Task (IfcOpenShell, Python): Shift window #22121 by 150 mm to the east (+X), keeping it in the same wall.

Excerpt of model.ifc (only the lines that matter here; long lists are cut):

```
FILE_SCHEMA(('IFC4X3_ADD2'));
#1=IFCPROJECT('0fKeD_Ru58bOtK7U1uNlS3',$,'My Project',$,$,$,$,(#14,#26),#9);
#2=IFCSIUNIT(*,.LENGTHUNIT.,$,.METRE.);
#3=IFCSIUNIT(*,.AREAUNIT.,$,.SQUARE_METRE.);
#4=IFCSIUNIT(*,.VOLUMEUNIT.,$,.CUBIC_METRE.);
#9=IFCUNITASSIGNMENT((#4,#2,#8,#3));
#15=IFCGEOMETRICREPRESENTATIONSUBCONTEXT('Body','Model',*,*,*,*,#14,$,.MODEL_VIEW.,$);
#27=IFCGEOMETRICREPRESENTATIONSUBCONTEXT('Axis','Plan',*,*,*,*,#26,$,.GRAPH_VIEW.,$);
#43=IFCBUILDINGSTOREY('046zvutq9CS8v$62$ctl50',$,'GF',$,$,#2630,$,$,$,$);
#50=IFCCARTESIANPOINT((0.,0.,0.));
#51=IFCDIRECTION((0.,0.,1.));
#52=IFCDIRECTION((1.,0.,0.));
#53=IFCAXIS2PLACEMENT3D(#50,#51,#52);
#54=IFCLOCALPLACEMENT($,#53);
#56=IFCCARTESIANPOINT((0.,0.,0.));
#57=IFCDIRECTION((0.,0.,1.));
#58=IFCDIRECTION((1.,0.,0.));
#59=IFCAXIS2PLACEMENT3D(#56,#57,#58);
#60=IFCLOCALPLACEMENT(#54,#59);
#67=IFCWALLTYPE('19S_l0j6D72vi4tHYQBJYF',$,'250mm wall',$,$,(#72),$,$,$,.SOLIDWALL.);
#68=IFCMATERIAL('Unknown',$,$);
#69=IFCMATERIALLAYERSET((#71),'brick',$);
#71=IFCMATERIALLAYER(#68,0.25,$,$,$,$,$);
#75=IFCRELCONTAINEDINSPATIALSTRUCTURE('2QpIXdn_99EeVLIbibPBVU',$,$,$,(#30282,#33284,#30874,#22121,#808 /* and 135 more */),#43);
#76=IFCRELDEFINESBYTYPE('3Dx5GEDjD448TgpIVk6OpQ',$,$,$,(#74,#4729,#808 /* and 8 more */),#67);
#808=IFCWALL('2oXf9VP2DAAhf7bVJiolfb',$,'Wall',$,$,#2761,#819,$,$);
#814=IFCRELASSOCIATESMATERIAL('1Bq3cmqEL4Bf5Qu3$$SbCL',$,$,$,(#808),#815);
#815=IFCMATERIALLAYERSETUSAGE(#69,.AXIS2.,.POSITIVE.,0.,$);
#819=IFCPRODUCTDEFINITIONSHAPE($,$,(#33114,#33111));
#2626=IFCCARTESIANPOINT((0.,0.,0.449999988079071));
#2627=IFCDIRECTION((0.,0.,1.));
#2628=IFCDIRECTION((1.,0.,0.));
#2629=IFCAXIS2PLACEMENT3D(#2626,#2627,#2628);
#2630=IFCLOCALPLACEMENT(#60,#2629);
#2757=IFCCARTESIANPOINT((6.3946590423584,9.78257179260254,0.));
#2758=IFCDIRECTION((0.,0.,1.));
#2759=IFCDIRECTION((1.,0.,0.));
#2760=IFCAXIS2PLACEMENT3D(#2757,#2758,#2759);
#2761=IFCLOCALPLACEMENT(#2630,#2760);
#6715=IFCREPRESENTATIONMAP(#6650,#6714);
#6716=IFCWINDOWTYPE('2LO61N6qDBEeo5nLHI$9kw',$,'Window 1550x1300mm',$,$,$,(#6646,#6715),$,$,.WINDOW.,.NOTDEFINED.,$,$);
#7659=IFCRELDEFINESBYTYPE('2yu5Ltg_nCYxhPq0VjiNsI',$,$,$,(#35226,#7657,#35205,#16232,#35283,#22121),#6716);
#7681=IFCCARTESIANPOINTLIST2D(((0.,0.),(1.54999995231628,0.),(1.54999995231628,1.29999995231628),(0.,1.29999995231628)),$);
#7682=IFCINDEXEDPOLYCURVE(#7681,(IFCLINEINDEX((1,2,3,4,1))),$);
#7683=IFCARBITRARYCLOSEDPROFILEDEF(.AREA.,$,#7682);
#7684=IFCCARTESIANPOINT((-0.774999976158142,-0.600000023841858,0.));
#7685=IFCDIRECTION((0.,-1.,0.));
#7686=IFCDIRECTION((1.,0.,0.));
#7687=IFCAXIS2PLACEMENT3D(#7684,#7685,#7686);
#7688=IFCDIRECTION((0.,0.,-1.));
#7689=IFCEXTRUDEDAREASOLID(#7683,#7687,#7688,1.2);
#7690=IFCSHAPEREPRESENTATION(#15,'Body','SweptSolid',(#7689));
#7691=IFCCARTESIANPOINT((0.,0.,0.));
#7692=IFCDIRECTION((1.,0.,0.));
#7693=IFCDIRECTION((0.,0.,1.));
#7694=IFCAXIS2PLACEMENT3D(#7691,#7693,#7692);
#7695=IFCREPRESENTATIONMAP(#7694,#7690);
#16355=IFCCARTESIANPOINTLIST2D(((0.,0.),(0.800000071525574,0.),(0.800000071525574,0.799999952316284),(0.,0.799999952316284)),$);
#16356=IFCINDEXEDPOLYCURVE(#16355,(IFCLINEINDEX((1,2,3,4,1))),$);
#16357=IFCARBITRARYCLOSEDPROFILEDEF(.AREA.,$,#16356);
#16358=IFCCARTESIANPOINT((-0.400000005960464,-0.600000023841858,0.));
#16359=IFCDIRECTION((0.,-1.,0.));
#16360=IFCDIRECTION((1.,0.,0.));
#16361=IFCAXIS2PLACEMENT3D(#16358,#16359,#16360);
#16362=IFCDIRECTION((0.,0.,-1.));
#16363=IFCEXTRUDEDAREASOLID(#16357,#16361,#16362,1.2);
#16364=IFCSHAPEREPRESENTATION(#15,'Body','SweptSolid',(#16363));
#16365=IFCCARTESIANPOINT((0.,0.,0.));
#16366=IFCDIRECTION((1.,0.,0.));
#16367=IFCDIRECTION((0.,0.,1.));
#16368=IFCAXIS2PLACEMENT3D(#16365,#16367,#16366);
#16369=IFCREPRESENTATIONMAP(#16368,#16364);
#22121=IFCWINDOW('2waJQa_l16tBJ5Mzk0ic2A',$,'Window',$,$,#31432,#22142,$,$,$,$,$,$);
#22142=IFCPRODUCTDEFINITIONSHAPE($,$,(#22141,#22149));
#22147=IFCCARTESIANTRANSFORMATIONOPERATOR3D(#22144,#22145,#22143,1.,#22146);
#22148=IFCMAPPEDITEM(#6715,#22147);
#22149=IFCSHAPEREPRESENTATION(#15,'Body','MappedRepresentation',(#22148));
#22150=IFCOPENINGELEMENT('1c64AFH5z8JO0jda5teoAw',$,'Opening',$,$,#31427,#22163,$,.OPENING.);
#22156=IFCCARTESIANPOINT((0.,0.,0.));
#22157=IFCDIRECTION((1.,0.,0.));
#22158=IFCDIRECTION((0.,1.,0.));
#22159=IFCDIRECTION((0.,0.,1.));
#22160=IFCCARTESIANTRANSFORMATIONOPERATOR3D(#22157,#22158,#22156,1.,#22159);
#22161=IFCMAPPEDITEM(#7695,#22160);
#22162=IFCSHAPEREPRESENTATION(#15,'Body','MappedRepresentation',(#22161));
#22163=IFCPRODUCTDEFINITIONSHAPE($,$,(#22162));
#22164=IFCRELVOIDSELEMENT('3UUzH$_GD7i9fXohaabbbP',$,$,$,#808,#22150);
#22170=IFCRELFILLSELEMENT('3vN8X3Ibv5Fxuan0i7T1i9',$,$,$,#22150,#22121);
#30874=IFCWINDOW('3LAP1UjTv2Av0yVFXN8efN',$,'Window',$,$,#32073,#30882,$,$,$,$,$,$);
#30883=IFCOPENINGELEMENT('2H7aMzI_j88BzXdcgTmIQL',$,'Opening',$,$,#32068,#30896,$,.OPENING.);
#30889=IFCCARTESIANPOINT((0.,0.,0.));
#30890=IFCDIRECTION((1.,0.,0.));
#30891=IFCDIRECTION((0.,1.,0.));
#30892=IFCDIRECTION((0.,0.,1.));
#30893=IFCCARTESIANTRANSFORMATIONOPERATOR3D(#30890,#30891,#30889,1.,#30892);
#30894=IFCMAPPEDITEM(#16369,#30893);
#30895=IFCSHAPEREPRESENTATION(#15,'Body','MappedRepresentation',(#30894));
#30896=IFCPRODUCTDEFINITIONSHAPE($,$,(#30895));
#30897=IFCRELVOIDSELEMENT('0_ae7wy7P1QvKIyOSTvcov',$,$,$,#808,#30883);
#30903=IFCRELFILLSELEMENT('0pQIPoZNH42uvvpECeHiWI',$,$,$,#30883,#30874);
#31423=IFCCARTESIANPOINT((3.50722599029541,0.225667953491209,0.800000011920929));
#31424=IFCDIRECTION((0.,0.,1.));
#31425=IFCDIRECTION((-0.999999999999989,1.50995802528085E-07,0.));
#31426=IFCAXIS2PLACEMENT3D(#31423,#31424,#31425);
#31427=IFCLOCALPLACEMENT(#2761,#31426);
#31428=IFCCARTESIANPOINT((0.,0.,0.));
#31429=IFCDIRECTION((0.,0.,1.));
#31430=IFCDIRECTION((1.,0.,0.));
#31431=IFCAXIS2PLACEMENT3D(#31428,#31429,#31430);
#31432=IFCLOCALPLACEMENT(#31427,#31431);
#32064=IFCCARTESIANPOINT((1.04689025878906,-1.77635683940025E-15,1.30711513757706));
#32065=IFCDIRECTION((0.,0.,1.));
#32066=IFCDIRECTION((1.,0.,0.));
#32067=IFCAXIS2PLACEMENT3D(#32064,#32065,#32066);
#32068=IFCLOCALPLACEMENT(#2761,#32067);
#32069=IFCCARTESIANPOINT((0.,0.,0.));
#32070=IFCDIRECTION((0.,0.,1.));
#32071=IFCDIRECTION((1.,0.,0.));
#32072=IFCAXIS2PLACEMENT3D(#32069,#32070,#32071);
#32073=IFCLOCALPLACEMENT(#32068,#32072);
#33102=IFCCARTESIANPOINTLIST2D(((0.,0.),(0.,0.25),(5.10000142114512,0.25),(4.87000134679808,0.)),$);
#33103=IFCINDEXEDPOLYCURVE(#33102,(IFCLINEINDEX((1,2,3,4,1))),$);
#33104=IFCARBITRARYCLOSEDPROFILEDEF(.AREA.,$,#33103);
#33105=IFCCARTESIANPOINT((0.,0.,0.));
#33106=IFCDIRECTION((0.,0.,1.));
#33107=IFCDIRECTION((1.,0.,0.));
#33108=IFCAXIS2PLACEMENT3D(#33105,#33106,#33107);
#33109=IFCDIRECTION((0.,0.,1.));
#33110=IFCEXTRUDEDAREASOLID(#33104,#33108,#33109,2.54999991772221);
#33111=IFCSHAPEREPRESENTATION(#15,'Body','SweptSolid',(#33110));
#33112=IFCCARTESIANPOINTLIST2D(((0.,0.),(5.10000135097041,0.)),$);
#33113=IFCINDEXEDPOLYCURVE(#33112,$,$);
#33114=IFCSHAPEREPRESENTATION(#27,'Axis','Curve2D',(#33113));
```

```python
import ifcopenshell
import ifcopenshell.api.geometry
import ifcopenshell.util.placement

model = ifcopenshell.open("model.ifc")

window = model.by_guid("2waJQa_l16tBJ5Mzk0ic2A")
opening = window.FillsVoids[0].RelatingOpeningElement
wall = opening.VoidsElements[0].RelatingBuildingElement

wall_matrix = ifcopenshell.util.placement.get_local_placement(wall.ObjectPlacement)
shift = wall_matrix[:3, 0] * 0.15
before = ifcopenshell.util.placement.get_local_placement(window.ObjectPlacement)[:3, 3].copy()

# The window is placed relative to its opening, so it follows when the opening moves.
matrix = ifcopenshell.util.placement.get_local_placement(opening.ObjectPlacement)
matrix[:3, 3] += shift
ifcopenshell.api.geometry.edit_object_placement(
    model, product=opening, matrix=matrix, is_si=False, should_transform_children=True
)

after = ifcopenshell.util.placement.get_local_placement(window.ObjectPlacement)[:3, 3]
print("window moved by", (after - before).round(3) + 0.0)

model.write("model-out.ifc")
```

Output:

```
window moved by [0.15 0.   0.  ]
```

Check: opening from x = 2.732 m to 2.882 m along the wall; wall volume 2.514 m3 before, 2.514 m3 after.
